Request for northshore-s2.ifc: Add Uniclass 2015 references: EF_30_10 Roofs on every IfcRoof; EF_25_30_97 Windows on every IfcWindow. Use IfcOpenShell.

First a look at what the model holds.

```python
import ifcopenshell

model = ifcopenshell.open("northshore-s2.ifc")
print(model.schema)
print("classifications:", [c.Name for c in model.by_type("IfcClassification")])
for ifc_class in ("IfcDoor", "IfcRoof", "IfcStair", "IfcWall", "IfcWindow"):
    print(ifc_class, len(model.by_type(ifc_class)))
```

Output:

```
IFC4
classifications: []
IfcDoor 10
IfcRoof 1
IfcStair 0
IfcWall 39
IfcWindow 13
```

```python
import ifcopenshell
import ifcopenshell.api.classification

model = ifcopenshell.open("northshore-s2.ifc")

system = ifcopenshell.api.classification.add_classification(model, classification="Uniclass 2015")

codes = {
    "IfcRoof": ("EF_30_10", "Roofs"),
    "IfcWindow": ("EF_25_30_97", "Windows"),
}
for ifc_class, (code, name) in codes.items():
    products = model.by_type(ifc_class)
    ifcopenshell.api.classification.add_reference(
        model, products=products, classification=system, identification=code, name=name
    )
    print(code, len(products))

model.write("northshore-s2_v2.ifc")
```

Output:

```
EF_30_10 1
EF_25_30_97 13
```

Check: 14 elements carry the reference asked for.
